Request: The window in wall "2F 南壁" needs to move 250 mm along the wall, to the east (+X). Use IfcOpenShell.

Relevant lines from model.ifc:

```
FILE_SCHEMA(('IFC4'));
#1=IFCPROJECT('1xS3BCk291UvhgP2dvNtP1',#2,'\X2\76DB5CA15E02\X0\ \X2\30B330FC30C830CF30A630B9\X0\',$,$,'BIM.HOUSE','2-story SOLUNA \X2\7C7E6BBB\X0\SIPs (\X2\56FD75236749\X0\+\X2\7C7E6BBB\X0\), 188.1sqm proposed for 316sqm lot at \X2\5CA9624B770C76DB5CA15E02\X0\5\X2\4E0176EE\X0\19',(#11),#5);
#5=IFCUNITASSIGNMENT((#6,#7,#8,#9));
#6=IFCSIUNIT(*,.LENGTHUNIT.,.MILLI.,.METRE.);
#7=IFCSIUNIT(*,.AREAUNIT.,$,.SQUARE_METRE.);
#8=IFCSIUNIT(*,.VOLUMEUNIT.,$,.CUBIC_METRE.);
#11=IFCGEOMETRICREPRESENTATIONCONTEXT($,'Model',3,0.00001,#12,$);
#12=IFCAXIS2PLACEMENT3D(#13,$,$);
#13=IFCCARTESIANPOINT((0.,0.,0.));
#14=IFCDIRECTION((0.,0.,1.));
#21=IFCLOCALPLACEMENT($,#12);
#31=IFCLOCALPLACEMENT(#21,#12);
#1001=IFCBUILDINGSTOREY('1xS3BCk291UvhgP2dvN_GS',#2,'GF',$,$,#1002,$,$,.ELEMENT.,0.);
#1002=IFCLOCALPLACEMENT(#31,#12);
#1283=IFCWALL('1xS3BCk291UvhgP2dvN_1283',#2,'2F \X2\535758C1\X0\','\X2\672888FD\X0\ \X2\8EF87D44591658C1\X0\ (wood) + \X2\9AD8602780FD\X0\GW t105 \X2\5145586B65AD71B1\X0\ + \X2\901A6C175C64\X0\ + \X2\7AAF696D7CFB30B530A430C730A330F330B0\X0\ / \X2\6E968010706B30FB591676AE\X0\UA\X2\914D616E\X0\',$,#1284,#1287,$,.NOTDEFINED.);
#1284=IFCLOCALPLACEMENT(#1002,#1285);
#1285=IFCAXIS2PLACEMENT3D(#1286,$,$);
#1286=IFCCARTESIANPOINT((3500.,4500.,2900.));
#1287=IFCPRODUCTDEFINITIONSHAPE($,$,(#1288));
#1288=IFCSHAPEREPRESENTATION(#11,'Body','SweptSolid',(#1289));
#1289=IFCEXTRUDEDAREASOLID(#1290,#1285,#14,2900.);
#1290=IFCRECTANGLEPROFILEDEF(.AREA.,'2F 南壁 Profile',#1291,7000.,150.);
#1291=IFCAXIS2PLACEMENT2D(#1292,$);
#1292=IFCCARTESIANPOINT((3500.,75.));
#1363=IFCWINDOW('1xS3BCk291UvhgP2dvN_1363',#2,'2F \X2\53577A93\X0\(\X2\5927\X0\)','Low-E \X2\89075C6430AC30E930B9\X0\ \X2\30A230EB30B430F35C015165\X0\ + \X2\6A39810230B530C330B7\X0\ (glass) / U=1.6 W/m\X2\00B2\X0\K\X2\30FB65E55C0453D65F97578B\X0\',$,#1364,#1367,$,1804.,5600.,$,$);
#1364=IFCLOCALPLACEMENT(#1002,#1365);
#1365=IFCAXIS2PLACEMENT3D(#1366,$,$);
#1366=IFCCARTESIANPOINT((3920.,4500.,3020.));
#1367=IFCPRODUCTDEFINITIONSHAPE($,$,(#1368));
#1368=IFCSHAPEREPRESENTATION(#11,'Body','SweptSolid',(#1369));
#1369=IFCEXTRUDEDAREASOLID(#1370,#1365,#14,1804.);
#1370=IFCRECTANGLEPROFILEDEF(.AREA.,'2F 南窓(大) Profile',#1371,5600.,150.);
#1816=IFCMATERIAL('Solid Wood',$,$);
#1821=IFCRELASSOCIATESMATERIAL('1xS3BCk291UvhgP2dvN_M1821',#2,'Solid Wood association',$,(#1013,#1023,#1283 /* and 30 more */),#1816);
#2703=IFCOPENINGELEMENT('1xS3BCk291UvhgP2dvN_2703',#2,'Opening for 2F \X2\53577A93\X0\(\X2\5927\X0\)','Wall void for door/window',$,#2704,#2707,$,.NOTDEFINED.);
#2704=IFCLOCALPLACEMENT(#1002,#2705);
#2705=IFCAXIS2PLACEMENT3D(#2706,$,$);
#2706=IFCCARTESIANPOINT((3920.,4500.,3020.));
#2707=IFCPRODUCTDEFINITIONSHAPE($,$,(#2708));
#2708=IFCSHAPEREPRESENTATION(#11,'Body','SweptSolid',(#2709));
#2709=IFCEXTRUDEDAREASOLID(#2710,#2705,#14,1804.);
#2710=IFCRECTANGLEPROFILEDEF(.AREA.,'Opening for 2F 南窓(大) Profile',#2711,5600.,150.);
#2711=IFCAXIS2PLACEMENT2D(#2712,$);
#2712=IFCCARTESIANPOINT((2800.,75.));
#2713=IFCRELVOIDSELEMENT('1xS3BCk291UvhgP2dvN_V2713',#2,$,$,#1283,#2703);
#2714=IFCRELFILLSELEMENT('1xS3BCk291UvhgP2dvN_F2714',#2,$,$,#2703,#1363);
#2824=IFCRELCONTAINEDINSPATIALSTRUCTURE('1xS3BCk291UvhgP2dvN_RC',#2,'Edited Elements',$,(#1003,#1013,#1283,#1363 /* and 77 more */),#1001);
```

```python
import ifcopenshell
import ifcopenshell.api.geometry
import ifcopenshell.util.placement
import ifcopenshell.util.unit

model = ifcopenshell.open("model.ifc")
unit_scale = ifcopenshell.util.unit.calculate_unit_scale(model)

window = model.by_id(1363)
opening = window.FillsVoids[0].RelatingOpeningElement
wall = opening.VoidsElements[0].RelatingBuildingElement

wall_matrix = ifcopenshell.util.placement.get_local_placement(wall.ObjectPlacement)
shift = wall_matrix[:3, 0] * 0.25 / unit_scale
before = ifcopenshell.util.placement.get_local_placement(window.ObjectPlacement)[:3, 3].copy()

# The window is not placed relative to its opening, so move both.
for product in (opening, window):
    matrix = ifcopenshell.util.placement.get_local_placement(product.ObjectPlacement)
    matrix[:3, 3] += shift
    ifcopenshell.api.geometry.edit_object_placement(model, product=product, matrix=matrix, is_si=False)

after = ifcopenshell.util.placement.get_local_placement(window.ObjectPlacement)[:3, 3]
print("window moved by", (after - before).round(3) + 0.0)

model.write("model-out.ifc")
```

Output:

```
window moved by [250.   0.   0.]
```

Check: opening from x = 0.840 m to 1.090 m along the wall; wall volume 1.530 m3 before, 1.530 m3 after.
